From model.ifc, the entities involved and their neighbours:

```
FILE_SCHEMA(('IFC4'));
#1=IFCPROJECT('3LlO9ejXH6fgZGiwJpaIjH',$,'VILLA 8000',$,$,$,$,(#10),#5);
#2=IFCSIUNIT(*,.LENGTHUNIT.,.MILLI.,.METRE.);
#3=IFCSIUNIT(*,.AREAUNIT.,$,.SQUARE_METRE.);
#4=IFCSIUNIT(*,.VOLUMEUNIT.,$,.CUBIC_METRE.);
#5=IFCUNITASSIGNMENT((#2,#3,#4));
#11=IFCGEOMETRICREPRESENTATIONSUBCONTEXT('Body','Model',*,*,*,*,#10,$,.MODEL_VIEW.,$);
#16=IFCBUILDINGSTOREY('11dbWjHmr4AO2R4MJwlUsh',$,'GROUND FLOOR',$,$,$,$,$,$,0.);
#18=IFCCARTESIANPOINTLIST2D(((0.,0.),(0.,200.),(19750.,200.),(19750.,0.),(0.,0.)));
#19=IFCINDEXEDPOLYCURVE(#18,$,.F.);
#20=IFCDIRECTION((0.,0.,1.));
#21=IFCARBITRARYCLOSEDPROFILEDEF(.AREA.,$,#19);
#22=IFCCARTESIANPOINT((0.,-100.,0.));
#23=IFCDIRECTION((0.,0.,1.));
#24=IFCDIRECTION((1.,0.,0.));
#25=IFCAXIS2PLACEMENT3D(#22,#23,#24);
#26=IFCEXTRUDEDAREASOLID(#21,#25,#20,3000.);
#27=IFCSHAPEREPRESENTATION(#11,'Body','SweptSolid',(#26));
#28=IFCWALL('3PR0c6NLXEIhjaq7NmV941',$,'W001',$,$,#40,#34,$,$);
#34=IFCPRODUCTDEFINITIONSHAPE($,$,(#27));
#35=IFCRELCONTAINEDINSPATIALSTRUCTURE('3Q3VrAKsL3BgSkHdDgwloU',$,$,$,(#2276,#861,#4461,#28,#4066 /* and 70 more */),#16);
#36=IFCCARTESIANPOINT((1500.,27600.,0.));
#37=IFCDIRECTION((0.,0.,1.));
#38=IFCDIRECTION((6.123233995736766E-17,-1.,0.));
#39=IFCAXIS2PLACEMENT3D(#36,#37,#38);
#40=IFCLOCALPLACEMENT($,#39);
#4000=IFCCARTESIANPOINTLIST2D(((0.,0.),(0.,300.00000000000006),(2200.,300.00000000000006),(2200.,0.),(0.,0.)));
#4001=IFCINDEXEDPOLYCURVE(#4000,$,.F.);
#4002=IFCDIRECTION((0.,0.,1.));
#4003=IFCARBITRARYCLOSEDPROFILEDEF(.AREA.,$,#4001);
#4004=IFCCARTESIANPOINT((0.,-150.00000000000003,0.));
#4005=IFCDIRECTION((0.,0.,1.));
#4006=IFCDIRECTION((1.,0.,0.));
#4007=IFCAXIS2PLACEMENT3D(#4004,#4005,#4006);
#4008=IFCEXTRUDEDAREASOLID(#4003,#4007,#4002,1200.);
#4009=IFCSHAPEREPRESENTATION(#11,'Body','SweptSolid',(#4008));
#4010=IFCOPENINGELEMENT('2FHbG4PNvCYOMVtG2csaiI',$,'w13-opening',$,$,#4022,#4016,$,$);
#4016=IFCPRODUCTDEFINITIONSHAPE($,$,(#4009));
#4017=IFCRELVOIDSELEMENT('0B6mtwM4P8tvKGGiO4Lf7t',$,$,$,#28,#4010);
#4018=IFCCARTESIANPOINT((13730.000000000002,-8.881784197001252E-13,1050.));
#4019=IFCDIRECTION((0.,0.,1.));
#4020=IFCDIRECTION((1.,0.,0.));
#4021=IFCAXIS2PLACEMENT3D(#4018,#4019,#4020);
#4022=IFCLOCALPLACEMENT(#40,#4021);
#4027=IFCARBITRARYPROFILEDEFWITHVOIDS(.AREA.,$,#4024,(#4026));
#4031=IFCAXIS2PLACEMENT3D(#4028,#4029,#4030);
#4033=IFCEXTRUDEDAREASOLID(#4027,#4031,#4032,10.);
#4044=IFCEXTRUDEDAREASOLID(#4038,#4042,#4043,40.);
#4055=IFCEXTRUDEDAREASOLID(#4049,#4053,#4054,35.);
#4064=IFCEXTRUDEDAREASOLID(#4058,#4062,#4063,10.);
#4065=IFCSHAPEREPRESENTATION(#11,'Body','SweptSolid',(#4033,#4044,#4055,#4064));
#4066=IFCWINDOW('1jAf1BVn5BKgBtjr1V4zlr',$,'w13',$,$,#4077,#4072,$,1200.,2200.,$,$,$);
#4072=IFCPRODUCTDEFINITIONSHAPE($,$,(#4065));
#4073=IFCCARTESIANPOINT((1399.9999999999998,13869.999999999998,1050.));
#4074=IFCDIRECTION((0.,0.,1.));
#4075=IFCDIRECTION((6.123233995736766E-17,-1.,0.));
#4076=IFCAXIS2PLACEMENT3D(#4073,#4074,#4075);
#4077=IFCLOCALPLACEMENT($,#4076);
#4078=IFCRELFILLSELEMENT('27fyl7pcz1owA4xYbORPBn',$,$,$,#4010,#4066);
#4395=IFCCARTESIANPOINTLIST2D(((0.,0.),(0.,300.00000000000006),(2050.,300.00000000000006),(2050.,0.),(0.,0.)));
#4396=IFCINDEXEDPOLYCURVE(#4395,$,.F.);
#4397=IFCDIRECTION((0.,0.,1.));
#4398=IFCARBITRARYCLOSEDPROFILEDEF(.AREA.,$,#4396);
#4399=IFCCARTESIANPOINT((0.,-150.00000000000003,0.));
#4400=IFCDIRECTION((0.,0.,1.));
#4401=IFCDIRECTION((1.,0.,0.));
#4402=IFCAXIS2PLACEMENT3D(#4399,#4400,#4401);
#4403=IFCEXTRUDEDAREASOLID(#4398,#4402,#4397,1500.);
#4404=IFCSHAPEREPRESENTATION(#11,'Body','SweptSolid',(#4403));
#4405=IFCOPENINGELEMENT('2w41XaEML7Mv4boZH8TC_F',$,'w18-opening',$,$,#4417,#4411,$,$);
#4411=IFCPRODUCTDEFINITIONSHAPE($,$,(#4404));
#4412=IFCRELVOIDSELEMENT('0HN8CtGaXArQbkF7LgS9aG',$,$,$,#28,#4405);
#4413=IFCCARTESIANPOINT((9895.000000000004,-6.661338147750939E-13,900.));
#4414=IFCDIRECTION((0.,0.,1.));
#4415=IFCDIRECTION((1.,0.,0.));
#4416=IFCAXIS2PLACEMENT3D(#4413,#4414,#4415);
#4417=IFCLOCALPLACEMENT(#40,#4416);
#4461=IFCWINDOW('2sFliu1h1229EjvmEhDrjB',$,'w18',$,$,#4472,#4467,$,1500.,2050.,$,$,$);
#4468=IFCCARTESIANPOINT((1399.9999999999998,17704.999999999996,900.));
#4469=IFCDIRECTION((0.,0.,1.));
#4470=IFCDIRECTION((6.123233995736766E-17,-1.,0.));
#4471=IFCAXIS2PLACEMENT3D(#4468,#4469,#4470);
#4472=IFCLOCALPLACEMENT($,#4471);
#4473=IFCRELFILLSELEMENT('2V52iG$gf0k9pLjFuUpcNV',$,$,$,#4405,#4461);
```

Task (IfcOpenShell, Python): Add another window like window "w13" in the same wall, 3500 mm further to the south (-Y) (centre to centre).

```python
import ifcopenshell
import ifcopenshell.api.feature
import ifcopenshell.api.geometry
import ifcopenshell.api.root
import ifcopenshell.geom
import ifcopenshell.util.element
import ifcopenshell.util.placement
import ifcopenshell.util.shape
import ifcopenshell.util.unit

model = ifcopenshell.open("model.ifc")
unit_scale = ifcopenshell.util.unit.calculate_unit_scale(model)
settings = ifcopenshell.geom.settings()


def volume(element):
    """Net volume in cubic metres, openings subtracted."""
    shape = ifcopenshell.geom.create_shape(settings, element)
    return ifcopenshell.util.shape.get_volume(shape.geometry)


window = model.by_guid("1jAf1BVn5BKgBtjr1V4zlr")
opening = window.FillsVoids[0].RelatingOpeningElement
wall = opening.VoidsElements[0].RelatingBuildingElement
before = volume(wall)
shift = ifcopenshell.util.placement.get_local_placement(wall.ObjectPlacement)[:3, 0] * 3.5 / unit_scale

# copy_class copies the void relationship, type, container and properties, but no geometry.
new_opening = ifcopenshell.api.root.copy_class(model, product=opening)
new_opening.Representation = ifcopenshell.util.element.copy_deep(
    model, opening.Representation, exclude=["IfcGeometricRepresentationContext", "IfcRepresentationMap"]
)
new_window = ifcopenshell.api.root.copy_class(model, product=window)
new_window.Representation = ifcopenshell.util.element.copy_deep(
    model, window.Representation, exclude=["IfcGeometricRepresentationContext", "IfcRepresentationMap"]
)
ifcopenshell.api.feature.add_filling(model, opening=new_opening, element=new_window)

for old, new in ((opening, new_opening), (window, new_window)):
    matrix = ifcopenshell.util.placement.get_local_placement(old.ObjectPlacement)
    matrix[:3, 3] += shift
    ifcopenshell.api.geometry.edit_object_placement(model, product=new, matrix=matrix, is_si=False)

after = volume(wall)

print(f"wall volume {before:.3f} -> {after:.3f} m3")

model.write("model-out.ifc")
```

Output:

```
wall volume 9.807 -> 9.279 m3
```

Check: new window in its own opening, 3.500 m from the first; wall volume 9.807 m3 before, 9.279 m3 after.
